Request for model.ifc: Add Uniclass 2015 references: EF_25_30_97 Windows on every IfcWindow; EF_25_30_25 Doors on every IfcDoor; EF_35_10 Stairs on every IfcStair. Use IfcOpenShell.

First a look at what the model holds.

```python
import ifcopenshell

model = ifcopenshell.open("model.ifc")
print(model.schema)
print("classifications:", [c.Name for c in model.by_type("IfcClassification")])
for ifc_class in ("IfcDoor", "IfcRoof", "IfcStair", "IfcWall", "IfcWindow"):
    print(ifc_class, len(model.by_type(ifc_class)))
```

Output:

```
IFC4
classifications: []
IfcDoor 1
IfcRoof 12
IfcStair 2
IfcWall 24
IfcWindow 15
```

```python
import ifcopenshell
import ifcopenshell.api.classification

model = ifcopenshell.open("model.ifc")

system = ifcopenshell.api.classification.add_classification(model, classification="Uniclass 2015")

codes = {
    "IfcWindow": ("EF_25_30_97", "Windows"),
    "IfcDoor": ("EF_25_30_25", "Doors"),
    "IfcStair": ("EF_35_10", "Stairs"),
}
for ifc_class, (code, name) in codes.items():
    products = model.by_type(ifc_class)
    ifcopenshell.api.classification.add_reference(
        model, products=products, classification=system, identification=code, name=name
    )
    print(code, len(products))

model.write("model_edited.ifc")
```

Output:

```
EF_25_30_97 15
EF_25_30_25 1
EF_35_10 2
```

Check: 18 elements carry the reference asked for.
